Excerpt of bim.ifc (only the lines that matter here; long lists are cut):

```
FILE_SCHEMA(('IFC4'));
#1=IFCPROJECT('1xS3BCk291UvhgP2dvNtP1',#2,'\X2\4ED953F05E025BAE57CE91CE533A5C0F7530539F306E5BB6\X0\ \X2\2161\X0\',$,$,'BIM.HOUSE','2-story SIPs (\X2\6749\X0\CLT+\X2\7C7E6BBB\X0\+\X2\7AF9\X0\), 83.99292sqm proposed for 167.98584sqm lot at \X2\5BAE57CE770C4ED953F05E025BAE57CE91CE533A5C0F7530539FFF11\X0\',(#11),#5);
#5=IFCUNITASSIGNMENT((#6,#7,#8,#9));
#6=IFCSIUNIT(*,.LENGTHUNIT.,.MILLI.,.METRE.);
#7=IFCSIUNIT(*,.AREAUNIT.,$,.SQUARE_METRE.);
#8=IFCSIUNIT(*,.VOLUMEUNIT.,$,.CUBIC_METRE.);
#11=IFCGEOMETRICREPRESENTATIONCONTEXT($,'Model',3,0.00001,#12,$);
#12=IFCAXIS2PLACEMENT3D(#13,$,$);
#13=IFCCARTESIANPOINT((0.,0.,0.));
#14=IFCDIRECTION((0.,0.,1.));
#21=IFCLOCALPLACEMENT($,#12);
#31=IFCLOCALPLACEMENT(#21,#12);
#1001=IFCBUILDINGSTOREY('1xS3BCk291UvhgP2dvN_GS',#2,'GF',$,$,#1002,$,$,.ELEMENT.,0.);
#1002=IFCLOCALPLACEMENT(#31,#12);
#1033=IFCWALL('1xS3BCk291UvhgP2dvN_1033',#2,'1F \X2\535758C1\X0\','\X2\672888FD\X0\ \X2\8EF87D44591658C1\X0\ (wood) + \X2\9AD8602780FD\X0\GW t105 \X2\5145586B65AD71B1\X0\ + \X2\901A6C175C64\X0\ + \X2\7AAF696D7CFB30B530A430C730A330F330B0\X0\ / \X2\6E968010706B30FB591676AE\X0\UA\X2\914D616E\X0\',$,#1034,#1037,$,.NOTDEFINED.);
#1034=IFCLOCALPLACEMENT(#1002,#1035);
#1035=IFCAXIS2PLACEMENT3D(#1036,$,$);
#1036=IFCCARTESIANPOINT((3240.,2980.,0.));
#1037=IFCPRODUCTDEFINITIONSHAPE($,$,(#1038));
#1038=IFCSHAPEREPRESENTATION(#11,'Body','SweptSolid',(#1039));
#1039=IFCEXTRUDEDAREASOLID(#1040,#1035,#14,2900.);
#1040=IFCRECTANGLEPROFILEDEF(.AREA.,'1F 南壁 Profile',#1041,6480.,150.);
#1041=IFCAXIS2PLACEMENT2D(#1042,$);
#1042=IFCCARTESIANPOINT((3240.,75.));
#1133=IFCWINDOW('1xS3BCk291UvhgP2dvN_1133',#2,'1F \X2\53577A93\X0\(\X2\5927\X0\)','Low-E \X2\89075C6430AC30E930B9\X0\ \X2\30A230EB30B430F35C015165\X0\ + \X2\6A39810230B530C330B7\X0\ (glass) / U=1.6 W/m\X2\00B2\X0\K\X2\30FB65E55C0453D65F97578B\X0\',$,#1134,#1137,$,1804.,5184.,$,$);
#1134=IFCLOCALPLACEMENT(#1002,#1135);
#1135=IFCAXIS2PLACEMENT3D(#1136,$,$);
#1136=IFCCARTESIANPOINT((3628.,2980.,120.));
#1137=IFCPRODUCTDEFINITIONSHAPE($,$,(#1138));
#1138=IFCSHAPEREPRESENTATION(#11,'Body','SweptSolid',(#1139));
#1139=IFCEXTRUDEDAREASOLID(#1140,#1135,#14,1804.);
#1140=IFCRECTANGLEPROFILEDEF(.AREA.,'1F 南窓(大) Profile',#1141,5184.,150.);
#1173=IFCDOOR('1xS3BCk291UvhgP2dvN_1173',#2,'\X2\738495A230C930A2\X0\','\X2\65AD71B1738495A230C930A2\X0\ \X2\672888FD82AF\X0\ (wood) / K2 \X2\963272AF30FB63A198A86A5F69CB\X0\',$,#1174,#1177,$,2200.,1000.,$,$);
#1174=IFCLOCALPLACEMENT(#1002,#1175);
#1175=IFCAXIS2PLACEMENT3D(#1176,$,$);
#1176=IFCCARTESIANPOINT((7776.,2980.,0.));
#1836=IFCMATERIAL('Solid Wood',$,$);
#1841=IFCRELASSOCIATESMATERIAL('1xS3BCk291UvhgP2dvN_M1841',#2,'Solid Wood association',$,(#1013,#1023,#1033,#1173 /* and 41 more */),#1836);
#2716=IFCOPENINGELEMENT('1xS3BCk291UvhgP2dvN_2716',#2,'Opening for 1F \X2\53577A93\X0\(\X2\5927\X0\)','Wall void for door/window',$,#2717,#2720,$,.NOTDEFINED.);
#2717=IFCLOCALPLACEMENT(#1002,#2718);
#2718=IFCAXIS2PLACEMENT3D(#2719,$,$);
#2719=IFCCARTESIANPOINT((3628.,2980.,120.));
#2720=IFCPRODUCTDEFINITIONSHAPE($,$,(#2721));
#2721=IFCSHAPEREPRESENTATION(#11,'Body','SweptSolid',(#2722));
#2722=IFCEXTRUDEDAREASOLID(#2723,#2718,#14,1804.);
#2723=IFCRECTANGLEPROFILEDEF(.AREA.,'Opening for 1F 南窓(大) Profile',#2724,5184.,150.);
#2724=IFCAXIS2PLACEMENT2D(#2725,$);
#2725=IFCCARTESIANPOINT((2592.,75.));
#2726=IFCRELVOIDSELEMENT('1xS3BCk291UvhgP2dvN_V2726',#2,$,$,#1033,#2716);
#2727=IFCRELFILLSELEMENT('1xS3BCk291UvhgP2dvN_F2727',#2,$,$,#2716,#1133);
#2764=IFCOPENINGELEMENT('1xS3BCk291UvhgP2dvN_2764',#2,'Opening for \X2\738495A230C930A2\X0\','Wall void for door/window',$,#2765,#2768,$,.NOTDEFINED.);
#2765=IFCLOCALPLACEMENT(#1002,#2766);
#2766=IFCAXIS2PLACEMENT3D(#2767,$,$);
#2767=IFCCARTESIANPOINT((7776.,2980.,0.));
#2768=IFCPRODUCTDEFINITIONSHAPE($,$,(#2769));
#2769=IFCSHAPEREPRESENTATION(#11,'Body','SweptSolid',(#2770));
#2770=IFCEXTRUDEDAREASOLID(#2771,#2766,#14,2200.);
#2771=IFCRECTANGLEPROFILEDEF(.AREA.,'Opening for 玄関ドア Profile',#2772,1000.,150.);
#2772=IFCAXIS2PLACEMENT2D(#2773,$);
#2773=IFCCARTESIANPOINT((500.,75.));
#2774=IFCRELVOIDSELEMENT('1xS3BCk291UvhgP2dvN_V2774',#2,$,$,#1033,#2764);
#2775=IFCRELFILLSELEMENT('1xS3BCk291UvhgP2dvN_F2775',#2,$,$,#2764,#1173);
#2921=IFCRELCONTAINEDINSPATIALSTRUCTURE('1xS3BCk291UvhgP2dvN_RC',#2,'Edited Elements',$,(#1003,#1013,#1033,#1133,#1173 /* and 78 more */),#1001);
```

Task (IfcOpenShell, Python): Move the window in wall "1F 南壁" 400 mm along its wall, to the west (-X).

```python
import ifcopenshell
import ifcopenshell.api.geometry
import ifcopenshell.util.placement

model = ifcopenshell.open("bim.ifc")

window = model.by_guid("1xS3BCk291UvhgP2dvN_1133")
opening = window.FillsVoids[0].RelatingOpeningElement
wall = opening.VoidsElements[0].RelatingBuildingElement

wall_matrix = ifcopenshell.util.placement.get_local_placement(wall.ObjectPlacement)
shift = wall_matrix[:3, 0] * -400.0
before = ifcopenshell.util.placement.get_local_placement(window.ObjectPlacement)[:3, 3].copy()

# The window is not placed relative to its opening, so move both.
for product in (opening, window):
    matrix = ifcopenshell.util.placement.get_local_placement(product.ObjectPlacement)
    matrix[:3, 3] += shift
    ifcopenshell.api.geometry.edit_object_placement(model, product=product, matrix=matrix, is_si=False)

after = ifcopenshell.util.placement.get_local_placement(window.ObjectPlacement)[:3, 3]
print("window moved by", (after - before).round(3) + 0.0)

model.write("bim_edited.ifc")
```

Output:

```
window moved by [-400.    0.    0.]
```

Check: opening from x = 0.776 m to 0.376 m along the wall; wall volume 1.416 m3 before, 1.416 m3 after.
